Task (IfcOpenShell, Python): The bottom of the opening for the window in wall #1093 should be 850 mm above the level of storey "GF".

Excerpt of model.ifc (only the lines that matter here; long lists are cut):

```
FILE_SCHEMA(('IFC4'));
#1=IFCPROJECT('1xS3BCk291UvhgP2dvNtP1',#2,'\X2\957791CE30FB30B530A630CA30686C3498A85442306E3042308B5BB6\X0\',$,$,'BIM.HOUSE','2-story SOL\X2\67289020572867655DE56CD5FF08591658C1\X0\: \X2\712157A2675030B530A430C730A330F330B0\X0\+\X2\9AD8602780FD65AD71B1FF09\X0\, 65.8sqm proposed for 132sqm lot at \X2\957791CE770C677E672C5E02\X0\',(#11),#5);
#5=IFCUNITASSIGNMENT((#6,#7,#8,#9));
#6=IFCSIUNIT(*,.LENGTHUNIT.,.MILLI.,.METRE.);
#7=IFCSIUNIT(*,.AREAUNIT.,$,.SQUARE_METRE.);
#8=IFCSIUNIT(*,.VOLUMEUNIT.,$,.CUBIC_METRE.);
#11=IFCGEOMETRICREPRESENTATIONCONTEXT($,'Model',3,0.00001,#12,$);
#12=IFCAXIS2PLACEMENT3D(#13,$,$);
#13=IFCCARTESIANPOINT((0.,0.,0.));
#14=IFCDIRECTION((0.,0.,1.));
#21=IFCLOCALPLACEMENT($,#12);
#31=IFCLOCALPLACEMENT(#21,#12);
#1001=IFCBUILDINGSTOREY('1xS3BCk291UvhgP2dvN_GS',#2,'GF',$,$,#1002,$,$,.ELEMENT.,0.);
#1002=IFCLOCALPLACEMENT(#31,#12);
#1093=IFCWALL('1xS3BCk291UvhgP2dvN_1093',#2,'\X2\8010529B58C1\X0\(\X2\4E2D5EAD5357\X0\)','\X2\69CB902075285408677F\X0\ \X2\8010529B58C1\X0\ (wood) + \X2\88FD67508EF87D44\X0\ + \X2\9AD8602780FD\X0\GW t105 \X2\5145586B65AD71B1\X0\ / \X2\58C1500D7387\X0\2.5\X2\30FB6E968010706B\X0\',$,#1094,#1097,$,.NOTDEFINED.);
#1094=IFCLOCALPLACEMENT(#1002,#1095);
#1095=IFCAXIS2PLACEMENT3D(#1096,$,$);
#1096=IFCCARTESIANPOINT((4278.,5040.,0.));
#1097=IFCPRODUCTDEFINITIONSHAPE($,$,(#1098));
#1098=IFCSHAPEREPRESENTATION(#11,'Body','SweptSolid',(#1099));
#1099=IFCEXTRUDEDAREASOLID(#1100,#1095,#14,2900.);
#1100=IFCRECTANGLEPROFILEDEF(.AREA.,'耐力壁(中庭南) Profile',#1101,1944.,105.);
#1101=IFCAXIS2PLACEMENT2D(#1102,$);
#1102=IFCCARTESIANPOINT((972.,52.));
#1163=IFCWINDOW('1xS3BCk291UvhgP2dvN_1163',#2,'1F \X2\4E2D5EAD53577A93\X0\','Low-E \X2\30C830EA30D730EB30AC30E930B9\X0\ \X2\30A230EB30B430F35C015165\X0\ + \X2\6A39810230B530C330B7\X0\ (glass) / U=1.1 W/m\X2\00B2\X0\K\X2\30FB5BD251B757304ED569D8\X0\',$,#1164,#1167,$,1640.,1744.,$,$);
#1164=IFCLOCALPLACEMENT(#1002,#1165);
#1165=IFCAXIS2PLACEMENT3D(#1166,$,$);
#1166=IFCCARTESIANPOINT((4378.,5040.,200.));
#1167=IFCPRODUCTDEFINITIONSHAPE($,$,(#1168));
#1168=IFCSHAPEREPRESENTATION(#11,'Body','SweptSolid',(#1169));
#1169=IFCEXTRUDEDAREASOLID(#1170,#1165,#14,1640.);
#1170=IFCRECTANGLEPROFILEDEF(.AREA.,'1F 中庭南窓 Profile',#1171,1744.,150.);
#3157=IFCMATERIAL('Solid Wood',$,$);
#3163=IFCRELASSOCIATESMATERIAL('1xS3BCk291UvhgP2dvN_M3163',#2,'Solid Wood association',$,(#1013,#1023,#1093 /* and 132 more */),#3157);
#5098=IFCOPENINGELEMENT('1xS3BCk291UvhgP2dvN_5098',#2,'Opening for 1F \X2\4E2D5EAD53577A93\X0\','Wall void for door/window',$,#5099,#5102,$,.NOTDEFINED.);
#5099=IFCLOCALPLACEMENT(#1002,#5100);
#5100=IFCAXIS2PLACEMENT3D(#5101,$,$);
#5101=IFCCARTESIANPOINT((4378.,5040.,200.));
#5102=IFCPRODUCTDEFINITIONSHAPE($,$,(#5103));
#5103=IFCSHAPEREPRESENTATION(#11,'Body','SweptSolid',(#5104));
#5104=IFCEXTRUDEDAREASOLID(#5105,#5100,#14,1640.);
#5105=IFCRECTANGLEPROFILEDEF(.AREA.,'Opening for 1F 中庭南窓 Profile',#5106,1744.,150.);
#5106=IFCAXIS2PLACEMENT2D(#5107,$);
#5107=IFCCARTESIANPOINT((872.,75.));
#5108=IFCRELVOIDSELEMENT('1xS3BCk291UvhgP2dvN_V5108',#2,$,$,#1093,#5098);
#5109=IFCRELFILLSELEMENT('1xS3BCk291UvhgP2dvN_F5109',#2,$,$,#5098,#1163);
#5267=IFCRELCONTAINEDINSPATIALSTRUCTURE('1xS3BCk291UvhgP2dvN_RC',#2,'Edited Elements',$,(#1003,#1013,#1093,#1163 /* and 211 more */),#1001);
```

```python
import numpy as np
import ifcopenshell
import ifcopenshell.api.geometry
import ifcopenshell.geom
import ifcopenshell.util.element
import ifcopenshell.util.placement
import ifcopenshell.util.shape
import ifcopenshell.util.unit

model = ifcopenshell.open("model.ifc")
unit_scale = ifcopenshell.util.unit.calculate_unit_scale(model)

window = model.by_guid("1xS3BCk291UvhgP2dvN_1163")
opening = window.FillsVoids[0].RelatingOpeningElement
storey = ifcopenshell.util.element.get_container(window, ifc_class="IfcBuildingStorey")
level = ifcopenshell.util.placement.get_local_placement(storey.ObjectPlacement)[2, 3]

# The opening's origin need not be at the sill, so measure its lowest point.
shape = ifcopenshell.geom.create_shape(ifcopenshell.geom.settings(), opening)
bottom = ifcopenshell.util.shape.get_shape_bottom_elevation(shape, shape.geometry) / unit_scale
dz = level + 0.85 / unit_scale - bottom

shift = np.array([0.0, 0.0, dz])
# The window is not placed relative to its opening, so move both.
for product in (opening, window):
    matrix = ifcopenshell.util.placement.get_local_placement(product.ObjectPlacement)
    matrix[:3, 3] += shift
    ifcopenshell.api.geometry.edit_object_placement(model, product=product, matrix=matrix, is_si=False)

print(f"moved by {dz * unit_scale:+.3f} m")

model.write("model_v2.ifc")
```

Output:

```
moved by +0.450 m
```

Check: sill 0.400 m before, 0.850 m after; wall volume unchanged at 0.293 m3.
